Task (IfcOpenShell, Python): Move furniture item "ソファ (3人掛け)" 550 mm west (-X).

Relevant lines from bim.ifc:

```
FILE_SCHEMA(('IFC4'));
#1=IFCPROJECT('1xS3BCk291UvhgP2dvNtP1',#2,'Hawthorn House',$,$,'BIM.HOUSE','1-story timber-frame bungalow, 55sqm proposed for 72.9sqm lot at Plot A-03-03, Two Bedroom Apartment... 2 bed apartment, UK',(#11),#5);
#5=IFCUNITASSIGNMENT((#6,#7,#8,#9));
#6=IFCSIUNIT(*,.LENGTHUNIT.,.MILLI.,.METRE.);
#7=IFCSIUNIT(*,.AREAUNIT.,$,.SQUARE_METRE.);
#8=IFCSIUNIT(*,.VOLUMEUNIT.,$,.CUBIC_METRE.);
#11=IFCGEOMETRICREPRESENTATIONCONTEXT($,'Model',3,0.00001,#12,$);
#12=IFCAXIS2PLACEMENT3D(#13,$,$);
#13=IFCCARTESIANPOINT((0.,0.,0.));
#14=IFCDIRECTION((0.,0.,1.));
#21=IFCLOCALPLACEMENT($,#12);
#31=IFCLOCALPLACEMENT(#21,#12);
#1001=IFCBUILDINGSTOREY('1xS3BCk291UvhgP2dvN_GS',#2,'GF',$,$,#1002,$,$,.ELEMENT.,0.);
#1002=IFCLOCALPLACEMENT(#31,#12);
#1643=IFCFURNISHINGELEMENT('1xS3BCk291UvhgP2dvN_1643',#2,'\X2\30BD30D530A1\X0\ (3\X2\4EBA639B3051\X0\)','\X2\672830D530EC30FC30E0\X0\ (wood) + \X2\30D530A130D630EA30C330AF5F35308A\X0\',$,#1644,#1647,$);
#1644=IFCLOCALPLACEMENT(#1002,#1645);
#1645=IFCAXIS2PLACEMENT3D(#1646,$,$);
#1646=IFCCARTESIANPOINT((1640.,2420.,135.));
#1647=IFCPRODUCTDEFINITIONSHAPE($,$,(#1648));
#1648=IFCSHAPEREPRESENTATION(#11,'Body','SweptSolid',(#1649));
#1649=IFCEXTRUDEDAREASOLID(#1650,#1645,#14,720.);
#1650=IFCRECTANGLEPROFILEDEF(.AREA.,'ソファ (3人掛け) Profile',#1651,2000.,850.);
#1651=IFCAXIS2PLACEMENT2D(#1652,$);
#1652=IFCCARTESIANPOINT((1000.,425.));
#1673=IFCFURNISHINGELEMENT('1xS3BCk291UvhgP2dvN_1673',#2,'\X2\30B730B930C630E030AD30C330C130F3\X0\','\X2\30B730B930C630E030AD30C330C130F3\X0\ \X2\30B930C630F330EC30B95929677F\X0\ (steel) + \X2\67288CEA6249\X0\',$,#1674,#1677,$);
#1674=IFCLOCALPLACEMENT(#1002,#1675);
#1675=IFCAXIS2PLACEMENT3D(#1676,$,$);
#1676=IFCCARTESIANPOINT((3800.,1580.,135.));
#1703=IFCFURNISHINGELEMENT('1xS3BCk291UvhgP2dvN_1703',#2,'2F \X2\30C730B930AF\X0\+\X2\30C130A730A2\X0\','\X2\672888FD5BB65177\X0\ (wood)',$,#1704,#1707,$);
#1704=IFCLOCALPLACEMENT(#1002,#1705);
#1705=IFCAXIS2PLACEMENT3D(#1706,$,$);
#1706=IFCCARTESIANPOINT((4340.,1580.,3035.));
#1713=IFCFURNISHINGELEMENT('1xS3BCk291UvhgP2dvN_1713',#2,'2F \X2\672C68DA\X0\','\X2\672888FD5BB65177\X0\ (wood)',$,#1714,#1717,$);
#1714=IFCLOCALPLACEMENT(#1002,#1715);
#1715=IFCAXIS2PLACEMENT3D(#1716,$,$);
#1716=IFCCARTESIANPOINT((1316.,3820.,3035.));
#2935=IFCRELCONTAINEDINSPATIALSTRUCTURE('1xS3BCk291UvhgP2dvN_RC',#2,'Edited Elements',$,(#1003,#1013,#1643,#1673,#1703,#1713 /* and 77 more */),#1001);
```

```python
import ifcopenshell
import ifcopenshell.api.geometry
import ifcopenshell.util.placement
import ifcopenshell.util.unit

model = ifcopenshell.open("bim.ifc")
unit_scale = ifcopenshell.util.unit.calculate_unit_scale(model)

item = model.by_id(1643)
matrix = ifcopenshell.util.placement.get_local_placement(item.ObjectPlacement)
matrix[0, 3] -= 0.55 / unit_scale
ifcopenshell.api.geometry.edit_object_placement(model, product=item, matrix=matrix, is_si=False)

print(ifcopenshell.util.placement.get_local_placement(item.ObjectPlacement).round(3) + 0.0)

model.write("bim_rev.ifc")
```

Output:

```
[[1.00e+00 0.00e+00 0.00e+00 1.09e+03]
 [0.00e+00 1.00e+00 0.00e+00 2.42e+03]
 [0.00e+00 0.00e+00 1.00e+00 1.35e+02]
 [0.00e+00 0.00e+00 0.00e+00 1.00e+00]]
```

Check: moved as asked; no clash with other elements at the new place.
